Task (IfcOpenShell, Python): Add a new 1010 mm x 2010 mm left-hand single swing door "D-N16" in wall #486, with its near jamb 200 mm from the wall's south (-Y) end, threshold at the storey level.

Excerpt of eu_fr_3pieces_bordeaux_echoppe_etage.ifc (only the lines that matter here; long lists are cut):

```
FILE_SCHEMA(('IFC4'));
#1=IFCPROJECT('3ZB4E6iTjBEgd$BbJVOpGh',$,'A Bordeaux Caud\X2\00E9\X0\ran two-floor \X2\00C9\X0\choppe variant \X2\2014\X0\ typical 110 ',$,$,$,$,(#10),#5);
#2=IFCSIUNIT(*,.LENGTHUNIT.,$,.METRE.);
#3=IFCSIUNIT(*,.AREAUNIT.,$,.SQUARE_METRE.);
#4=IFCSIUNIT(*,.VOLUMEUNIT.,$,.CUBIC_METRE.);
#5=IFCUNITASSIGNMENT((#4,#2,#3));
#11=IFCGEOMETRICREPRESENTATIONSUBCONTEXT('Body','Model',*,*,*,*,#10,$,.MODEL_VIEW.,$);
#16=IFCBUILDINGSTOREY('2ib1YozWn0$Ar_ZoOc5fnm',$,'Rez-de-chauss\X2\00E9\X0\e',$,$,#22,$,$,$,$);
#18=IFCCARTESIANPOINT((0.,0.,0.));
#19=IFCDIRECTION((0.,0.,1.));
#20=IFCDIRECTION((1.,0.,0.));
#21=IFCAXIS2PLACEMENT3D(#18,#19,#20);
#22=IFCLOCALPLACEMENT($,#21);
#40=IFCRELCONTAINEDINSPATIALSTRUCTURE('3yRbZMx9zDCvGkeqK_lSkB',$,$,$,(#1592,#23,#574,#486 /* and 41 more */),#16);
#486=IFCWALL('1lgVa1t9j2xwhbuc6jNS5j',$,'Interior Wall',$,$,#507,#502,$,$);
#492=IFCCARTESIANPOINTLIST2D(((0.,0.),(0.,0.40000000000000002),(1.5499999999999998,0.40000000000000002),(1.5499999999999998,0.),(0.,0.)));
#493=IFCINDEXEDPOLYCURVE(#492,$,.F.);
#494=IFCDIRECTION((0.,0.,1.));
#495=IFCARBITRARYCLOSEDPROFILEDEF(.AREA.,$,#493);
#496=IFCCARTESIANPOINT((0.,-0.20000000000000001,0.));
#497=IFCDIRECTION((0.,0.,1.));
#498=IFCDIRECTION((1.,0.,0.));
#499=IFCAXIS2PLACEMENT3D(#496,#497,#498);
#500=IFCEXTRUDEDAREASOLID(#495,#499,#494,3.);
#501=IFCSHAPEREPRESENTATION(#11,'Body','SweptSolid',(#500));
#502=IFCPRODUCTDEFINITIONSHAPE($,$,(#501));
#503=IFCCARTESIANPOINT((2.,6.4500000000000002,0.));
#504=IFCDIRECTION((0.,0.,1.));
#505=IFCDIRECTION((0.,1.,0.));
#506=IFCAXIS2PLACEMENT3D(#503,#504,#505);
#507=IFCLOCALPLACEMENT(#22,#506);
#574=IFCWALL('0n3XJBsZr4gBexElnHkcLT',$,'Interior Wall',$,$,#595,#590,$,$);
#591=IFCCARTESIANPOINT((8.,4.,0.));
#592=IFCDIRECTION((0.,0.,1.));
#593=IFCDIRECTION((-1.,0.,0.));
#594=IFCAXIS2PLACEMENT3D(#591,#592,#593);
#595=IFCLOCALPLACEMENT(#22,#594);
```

```python
import numpy as np
import ifcopenshell
import ifcopenshell.api.feature
import ifcopenshell.api.geometry
import ifcopenshell.api.root
import ifcopenshell.api.spatial
import ifcopenshell.geom
import ifcopenshell.util.element
import ifcopenshell.util.placement
import ifcopenshell.util.representation
import ifcopenshell.util.shape
import ifcopenshell.util.unit

model = ifcopenshell.open("eu_fr_3pieces_bordeaux_echoppe_etage.ifc")
unit_scale = ifcopenshell.util.unit.calculate_unit_scale(model)
settings = ifcopenshell.geom.settings()


def volume(element):
    """Net volume in cubic metres, openings subtracted."""
    shape = ifcopenshell.geom.create_shape(settings, element)
    return ifcopenshell.util.shape.get_volume(shape.geometry)


wall = model.by_guid("1lgVa1t9j2xwhbuc6jNS5j")
storey = ifcopenshell.util.element.get_container(wall, ifc_class="IfcBuildingStorey")
context = ifcopenshell.util.representation.get_context(model, "Model", "Body", "MODEL_VIEW")
before = volume(wall)

width, height, from_end, sill = 1.01, 2.01, 0.2, 0.0  # metres

# The wall runs along its own X axis, and the end named is its -X end.
wall_shape = ifcopenshell.geom.create_shape(settings, wall)
x, y, z = ifcopenshell.util.shape.get_vertices(wall_shape.geometry).T
start = x.min() + from_end
face, thickness = float(y.min()), float(y.max() - y.min())
wall_matrix = ifcopenshell.util.placement.get_local_placement(wall.ObjectPlacement)
level = ifcopenshell.util.placement.get_local_placement(storey.ObjectPlacement)[2, 3]


def in_wall(x, y):
    """Placement at x, y metres in the wall's axes, at sill height."""
    matrix = wall_matrix.copy()
    matrix[:, 3] = wall_matrix @ np.array([x / unit_scale, y / unit_scale, 0.0, 1.0])
    matrix[2, 3] = level + sill / unit_scale
    return matrix


# Opening: a box that overshoots both wall faces by 50 mm.
opening = ifcopenshell.api.root.create_entity(model, ifc_class="IfcOpeningElement", predefined_type="OPENING")
box = ifcopenshell.api.geometry.add_wall_representation(
    model, context=context, length=width, height=height, thickness=thickness + 0.1
)
ifcopenshell.api.geometry.assign_representation(model, product=opening, representation=box)
ifcopenshell.api.geometry.edit_object_placement(model, product=opening, matrix=in_wall(start, face - 0.05), is_si=False)
ifcopenshell.api.feature.add_feature(model, feature=opening, element=wall)

door = ifcopenshell.api.root.create_entity(model, ifc_class="IfcDoor", name="D-N16", predefined_type="DOOR")
door.OverallWidth, door.OverallHeight = width / unit_scale, height / unit_scale
door.OperationType = "SINGLE_SWING_LEFT"
body = ifcopenshell.api.geometry.add_door_representation(
    model,
    context=context,
    overall_width=door.OverallWidth,
    overall_height=door.OverallHeight,
    operation_type="SINGLE_SWING_LEFT",
    lining_properties={"LiningDepth": thickness / unit_scale, "ThresholdDepth": thickness / unit_scale},
)
ifcopenshell.api.geometry.assign_representation(model, product=door, representation=body)
ifcopenshell.api.spatial.assign_container(model, products=[door], relating_structure=storey)
ifcopenshell.api.feature.add_filling(model, opening=opening, element=door)

# The lining spans the wall, so the door starts at the wall face.
ifcopenshell.api.geometry.edit_object_placement(model, product=door, matrix=in_wall(start, face), is_si=False)

after = volume(wall)

print(f"wall volume {before:.3f} -> {after:.3f} m3")

model.write("eu_fr_3pieces_bordeaux_echoppe_etage_rev.ifc")
```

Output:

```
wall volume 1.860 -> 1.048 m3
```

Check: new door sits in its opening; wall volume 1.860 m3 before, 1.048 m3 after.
